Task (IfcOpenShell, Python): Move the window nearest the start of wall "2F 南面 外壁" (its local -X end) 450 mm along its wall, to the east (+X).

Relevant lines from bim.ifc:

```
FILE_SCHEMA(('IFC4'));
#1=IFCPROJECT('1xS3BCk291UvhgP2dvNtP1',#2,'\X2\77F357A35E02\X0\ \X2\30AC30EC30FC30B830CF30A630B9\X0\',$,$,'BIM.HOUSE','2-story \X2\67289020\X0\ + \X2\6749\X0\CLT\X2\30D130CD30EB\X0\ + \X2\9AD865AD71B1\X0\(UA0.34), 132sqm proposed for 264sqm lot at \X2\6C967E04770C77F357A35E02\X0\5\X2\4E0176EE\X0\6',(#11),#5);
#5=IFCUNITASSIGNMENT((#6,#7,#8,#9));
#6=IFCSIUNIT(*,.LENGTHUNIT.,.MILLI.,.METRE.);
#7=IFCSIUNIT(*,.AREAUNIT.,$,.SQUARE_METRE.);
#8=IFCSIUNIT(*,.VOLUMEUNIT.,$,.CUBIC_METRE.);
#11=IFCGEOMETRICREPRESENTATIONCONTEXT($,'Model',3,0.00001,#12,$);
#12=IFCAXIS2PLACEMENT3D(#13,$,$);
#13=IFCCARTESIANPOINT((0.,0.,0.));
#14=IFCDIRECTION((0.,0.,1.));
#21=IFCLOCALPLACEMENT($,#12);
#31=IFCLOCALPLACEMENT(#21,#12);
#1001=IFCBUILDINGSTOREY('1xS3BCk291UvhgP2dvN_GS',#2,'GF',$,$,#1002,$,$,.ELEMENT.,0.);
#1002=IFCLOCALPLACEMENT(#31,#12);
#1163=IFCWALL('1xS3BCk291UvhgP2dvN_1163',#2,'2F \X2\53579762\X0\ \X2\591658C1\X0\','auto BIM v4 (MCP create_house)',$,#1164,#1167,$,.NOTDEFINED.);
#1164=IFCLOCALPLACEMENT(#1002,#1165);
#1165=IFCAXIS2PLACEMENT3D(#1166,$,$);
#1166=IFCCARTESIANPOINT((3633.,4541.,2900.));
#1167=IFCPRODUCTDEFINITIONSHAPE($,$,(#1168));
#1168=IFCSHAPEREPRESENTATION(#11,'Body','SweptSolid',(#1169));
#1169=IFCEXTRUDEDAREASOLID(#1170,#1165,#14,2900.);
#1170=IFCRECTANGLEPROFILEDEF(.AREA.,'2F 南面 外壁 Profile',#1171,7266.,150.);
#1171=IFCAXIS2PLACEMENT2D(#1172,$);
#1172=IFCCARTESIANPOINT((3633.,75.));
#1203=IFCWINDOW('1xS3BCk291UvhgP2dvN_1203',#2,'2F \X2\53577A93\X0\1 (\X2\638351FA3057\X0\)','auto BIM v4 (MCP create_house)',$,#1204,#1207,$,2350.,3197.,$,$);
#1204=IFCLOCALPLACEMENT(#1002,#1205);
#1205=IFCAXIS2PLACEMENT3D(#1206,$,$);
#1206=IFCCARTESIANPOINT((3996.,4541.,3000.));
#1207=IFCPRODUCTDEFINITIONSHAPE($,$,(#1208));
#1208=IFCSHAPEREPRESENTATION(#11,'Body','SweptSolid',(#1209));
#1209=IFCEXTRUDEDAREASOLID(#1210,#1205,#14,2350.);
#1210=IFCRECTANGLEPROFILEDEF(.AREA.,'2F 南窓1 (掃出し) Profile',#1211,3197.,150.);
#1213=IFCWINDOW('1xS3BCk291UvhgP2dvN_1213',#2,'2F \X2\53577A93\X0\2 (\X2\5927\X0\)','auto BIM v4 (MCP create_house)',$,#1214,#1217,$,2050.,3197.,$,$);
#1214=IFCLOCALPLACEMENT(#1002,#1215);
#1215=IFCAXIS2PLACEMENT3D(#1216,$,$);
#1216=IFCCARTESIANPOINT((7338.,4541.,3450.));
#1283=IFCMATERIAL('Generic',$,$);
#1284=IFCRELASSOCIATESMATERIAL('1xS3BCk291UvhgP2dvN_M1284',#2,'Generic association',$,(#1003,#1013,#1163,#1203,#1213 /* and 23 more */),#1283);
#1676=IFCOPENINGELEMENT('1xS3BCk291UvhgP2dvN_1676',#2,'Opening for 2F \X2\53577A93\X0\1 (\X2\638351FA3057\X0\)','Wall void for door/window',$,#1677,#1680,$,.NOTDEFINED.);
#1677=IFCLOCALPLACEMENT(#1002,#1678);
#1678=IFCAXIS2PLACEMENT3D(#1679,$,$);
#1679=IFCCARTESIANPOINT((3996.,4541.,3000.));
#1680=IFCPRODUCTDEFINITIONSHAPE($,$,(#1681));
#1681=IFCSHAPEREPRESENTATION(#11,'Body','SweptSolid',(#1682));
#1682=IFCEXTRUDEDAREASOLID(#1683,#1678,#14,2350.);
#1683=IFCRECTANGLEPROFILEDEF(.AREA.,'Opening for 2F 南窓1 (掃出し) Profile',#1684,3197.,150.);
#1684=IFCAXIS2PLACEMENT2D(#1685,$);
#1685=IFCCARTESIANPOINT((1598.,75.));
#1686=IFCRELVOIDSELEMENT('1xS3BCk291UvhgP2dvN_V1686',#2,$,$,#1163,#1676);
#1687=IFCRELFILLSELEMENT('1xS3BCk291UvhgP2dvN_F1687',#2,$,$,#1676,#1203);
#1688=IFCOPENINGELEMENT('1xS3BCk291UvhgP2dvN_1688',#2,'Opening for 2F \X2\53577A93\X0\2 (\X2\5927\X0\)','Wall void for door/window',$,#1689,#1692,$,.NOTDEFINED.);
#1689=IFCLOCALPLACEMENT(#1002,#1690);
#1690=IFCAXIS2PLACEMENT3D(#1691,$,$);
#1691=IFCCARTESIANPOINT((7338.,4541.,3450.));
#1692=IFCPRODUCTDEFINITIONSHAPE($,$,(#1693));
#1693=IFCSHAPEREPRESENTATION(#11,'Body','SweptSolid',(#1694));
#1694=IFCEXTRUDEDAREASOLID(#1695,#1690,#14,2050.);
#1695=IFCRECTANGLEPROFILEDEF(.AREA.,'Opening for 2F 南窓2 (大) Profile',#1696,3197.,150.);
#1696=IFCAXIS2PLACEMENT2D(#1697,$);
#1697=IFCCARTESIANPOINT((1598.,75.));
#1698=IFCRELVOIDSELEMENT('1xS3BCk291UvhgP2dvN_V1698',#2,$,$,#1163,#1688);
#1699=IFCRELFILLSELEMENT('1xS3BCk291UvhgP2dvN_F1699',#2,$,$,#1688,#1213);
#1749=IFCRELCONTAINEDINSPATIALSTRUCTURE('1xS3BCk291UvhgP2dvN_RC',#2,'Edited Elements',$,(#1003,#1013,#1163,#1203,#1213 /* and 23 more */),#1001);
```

```python
import ifcopenshell
import ifcopenshell.api.geometry
import ifcopenshell.util.placement

model = ifcopenshell.open("bim.ifc")

window = model.by_guid("1xS3BCk291UvhgP2dvN_1203")
opening = window.FillsVoids[0].RelatingOpeningElement
wall = opening.VoidsElements[0].RelatingBuildingElement

wall_matrix = ifcopenshell.util.placement.get_local_placement(wall.ObjectPlacement)
shift = wall_matrix[:3, 0] * 450.0
before = ifcopenshell.util.placement.get_local_placement(window.ObjectPlacement)[:3, 3].copy()

# The window is not placed relative to its opening, so move both.
for product in (opening, window):
    matrix = ifcopenshell.util.placement.get_local_placement(product.ObjectPlacement)
    matrix[:3, 3] += shift
    ifcopenshell.api.geometry.edit_object_placement(model, product=product, matrix=matrix, is_si=False)

after = ifcopenshell.util.placement.get_local_placement(window.ObjectPlacement)[:3, 3]
print("window moved by", (after - before).round(3) + 0.0)

model.write("bim_edited.ifc")
```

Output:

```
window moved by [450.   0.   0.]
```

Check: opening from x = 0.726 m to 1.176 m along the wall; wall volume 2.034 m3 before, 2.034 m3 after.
